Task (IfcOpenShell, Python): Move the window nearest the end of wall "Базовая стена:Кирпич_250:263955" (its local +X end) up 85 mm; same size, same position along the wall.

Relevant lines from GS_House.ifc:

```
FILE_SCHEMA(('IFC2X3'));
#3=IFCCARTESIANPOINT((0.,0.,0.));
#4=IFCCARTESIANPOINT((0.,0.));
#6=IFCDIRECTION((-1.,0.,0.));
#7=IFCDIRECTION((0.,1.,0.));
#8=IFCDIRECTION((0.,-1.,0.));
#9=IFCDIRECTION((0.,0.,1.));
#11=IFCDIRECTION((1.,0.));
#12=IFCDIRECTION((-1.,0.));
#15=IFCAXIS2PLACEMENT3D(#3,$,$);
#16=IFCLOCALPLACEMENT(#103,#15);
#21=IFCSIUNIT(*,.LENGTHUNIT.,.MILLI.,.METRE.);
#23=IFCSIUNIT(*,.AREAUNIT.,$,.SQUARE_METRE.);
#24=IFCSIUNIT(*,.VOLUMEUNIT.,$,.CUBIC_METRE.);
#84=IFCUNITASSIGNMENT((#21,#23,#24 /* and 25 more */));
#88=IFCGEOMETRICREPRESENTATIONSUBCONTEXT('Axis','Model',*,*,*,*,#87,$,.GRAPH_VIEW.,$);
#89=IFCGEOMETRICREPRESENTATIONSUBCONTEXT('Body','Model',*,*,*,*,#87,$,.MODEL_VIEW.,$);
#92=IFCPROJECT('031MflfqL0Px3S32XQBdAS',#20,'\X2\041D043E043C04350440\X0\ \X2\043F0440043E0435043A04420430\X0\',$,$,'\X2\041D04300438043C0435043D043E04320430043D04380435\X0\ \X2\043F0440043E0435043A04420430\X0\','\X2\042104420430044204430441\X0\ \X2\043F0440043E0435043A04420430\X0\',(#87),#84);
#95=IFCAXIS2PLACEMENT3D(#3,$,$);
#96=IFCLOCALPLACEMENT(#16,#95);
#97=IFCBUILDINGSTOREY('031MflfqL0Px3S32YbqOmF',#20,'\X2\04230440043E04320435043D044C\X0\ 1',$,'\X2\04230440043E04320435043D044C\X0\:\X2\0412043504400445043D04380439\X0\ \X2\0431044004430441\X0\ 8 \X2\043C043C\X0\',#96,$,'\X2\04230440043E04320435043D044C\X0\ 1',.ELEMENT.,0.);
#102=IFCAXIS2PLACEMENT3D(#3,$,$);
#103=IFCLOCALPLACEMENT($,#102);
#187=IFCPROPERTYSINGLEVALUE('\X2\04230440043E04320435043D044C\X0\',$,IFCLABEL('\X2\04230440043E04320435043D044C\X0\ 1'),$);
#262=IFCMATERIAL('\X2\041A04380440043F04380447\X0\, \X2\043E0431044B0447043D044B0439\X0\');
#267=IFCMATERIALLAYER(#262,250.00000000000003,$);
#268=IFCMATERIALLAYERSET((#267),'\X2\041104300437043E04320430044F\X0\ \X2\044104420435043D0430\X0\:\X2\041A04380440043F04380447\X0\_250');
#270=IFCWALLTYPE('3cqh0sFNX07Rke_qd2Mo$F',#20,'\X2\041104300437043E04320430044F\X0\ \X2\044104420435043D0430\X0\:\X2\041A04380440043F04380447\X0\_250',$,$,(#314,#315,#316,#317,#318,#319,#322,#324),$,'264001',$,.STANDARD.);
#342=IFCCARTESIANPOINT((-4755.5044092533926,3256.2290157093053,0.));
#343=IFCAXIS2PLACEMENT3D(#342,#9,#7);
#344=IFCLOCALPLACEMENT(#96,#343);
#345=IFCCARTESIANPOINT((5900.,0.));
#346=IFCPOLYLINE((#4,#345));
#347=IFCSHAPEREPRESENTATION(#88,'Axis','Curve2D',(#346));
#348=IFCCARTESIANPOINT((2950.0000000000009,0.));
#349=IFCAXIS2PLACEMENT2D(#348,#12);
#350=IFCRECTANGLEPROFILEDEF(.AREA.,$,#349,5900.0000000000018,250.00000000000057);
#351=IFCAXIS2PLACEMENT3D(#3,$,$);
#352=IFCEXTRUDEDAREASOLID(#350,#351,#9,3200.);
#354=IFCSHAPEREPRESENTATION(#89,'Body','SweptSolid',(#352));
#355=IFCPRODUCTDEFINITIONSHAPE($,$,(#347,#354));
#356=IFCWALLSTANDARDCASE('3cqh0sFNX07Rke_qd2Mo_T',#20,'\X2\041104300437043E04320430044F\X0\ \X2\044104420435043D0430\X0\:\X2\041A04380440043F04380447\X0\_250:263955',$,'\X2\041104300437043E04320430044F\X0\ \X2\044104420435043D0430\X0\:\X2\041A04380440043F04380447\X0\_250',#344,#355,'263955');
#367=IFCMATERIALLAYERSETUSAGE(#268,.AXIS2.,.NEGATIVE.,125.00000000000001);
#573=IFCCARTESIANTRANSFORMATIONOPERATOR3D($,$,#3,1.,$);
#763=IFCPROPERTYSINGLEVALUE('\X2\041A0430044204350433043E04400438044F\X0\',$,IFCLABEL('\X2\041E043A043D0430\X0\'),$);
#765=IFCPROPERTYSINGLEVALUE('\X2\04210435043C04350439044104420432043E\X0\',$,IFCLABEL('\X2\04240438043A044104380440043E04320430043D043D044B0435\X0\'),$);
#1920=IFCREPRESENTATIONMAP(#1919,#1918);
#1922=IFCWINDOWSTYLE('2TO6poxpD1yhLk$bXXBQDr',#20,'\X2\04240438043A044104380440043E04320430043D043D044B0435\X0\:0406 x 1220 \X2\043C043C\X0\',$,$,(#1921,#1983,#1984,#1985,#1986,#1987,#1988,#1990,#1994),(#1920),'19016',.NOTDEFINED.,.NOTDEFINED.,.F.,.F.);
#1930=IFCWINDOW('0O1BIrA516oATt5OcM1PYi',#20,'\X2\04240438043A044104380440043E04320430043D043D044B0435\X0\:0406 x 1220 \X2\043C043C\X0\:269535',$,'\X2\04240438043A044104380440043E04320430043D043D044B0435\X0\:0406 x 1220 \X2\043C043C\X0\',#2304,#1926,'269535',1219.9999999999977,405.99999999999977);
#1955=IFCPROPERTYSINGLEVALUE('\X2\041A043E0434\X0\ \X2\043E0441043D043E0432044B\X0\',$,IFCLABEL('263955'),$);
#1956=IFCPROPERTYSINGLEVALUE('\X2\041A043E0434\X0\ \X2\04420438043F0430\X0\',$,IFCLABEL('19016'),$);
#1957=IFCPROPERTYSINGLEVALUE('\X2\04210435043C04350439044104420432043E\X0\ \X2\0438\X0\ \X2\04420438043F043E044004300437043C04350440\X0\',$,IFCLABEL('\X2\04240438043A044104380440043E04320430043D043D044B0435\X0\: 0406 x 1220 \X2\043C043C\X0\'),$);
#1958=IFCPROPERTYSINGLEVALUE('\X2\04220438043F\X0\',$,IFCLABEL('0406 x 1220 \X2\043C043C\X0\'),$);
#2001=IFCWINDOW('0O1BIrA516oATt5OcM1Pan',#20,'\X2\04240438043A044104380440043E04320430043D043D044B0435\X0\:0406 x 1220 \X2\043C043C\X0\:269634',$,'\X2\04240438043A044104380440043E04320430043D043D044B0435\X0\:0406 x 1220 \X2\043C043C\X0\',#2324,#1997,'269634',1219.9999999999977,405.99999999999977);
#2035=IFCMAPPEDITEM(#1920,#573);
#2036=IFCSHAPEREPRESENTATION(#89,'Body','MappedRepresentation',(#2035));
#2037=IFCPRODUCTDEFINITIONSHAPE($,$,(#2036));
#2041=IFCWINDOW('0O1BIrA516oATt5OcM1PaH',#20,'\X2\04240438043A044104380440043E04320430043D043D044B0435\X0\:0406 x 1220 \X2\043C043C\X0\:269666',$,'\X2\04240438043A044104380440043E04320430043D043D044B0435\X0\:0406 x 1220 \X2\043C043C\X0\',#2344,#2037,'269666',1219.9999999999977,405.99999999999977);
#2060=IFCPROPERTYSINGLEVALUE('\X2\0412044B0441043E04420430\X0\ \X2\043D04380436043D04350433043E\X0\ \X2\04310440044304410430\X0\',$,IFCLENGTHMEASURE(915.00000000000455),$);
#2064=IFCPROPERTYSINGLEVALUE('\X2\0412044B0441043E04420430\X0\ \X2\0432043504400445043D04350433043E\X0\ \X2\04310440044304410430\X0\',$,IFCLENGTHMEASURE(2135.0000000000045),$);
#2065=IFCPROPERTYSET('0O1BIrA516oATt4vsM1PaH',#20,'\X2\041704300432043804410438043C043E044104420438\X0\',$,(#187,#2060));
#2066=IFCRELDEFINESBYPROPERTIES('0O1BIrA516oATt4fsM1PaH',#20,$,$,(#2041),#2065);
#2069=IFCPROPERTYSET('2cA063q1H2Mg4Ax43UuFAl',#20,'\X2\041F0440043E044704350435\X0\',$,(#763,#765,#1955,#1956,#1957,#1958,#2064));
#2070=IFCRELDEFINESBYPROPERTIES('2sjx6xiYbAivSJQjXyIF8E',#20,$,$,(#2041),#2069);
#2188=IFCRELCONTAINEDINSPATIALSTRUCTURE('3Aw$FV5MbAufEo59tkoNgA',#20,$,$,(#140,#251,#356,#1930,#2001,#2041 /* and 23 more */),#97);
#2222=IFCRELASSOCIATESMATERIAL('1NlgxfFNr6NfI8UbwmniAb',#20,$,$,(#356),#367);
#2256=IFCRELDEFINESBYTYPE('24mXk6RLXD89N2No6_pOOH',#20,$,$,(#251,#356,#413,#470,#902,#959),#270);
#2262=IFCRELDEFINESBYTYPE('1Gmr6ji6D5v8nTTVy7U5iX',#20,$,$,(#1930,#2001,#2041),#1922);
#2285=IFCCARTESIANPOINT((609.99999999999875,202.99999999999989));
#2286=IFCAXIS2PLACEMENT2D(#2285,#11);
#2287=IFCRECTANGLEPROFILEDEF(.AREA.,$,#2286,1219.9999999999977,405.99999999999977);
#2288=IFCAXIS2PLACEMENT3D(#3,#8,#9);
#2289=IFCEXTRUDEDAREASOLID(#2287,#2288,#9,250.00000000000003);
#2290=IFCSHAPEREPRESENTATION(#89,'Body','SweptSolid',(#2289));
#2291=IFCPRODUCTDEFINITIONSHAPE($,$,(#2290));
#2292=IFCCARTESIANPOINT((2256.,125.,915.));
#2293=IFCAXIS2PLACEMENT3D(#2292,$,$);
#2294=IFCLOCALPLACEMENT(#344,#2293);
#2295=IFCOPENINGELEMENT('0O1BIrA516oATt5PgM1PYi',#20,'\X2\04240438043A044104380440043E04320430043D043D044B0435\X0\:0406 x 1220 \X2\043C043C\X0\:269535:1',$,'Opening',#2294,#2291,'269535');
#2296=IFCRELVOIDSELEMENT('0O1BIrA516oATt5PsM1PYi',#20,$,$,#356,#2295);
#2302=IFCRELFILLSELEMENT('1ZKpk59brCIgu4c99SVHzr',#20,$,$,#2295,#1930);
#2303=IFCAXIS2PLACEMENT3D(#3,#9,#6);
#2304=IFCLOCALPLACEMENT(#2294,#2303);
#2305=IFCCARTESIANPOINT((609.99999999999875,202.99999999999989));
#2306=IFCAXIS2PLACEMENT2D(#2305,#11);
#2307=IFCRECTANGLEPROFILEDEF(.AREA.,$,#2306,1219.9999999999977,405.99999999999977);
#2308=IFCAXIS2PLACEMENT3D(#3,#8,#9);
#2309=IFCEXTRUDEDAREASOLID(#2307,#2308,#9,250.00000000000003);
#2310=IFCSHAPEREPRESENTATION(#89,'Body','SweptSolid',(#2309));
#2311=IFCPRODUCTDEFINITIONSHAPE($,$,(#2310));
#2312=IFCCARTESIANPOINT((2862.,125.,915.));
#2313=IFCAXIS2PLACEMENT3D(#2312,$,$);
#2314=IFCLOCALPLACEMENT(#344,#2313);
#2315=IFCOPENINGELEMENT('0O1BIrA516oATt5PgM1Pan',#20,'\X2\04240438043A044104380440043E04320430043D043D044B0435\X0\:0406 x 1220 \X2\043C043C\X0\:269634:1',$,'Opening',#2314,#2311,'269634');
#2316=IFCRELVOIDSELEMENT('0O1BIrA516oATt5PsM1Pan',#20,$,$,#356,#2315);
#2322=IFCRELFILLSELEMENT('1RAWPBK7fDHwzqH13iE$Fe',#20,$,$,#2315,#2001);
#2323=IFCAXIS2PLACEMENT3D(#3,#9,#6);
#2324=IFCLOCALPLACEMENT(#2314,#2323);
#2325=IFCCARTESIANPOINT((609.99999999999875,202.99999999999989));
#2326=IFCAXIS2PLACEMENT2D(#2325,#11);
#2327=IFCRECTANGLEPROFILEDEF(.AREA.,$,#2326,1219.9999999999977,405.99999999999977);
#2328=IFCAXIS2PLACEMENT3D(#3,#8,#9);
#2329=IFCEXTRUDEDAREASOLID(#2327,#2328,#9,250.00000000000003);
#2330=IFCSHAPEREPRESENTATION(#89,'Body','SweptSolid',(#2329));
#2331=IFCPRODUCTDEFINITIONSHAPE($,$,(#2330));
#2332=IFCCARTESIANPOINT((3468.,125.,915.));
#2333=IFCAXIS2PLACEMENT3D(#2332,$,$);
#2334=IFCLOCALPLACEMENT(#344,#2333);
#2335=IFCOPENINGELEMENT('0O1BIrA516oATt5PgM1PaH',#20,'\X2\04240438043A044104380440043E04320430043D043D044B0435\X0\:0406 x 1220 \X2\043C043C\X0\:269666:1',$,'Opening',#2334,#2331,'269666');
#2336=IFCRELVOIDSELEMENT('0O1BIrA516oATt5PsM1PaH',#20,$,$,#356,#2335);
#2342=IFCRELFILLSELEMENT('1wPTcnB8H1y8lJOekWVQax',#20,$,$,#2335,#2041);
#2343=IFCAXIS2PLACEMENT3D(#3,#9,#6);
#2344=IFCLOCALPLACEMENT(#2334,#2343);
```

```python
import numpy as np
import ifcopenshell
import ifcopenshell.api.geometry
import ifcopenshell.api.pset
import ifcopenshell.util.element
import ifcopenshell.util.placement
import ifcopenshell.util.unit

model = ifcopenshell.open("GS_House.ifc")
unit_scale = ifcopenshell.util.unit.calculate_unit_scale(model)

window = model.by_guid("0O1BIrA516oATt5OcM1PaH")
opening = window.FillsVoids[0].RelatingOpeningElement
dz = 85.0

shift = np.array([0.0, 0.0, dz])
# The window is placed relative to its opening, so it follows when the opening moves.
matrix = ifcopenshell.util.placement.get_local_placement(opening.ObjectPlacement)
matrix[:3, 3] += shift
ifcopenshell.api.geometry.edit_object_placement(
    model, product=opening, matrix=matrix, is_si=False, should_transform_children=True
)

# Keep the stored heights in step.
pset = model.by_id(ifcopenshell.util.element.get_pset(window, "Зависимости", should_inherit=False)["id"])
ifcopenshell.api.pset.edit_pset(model, pset=pset, properties={
    "Высота нижнего бруса": model.create_entity("IfcLengthMeasure", ifcopenshell.util.element.get_pset(window, "Зависимости", "Высота нижнего бруса") + dz),
})
pset = model.by_id(ifcopenshell.util.element.get_pset(window, "Прочее", should_inherit=False)["id"])
ifcopenshell.api.pset.edit_pset(model, pset=pset, properties={
    "Высота верхнего бруса": model.create_entity("IfcLengthMeasure", ifcopenshell.util.element.get_pset(window, "Прочее", "Высота верхнего бруса") + dz),
})

print(f"moved by {dz * unit_scale:+.3f} m")

model.write("GS_House_rev.ifc")
```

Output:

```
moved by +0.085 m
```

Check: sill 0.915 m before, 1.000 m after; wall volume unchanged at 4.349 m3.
